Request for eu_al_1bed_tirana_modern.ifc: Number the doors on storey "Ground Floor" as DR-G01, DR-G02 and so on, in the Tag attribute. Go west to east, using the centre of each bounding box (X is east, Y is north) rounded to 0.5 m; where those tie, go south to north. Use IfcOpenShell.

First a look at what the model holds.

```python
import ifcopenshell
import ifcopenshell.util.element
import ifcopenshell.util.placement

model = ifcopenshell.open("eu_al_1bed_tirana_modern.ifc")
print(model.schema)
storey = next(s for s in model.by_type("IfcBuildingStorey") if s.Name == "Ground Floor")
doors = [e for e in ifcopenshell.util.element.get_decomposition(storey) if e.is_a("IfcDoor")]
for e in sorted(doors, key=lambda e: e.id()):
    origin = ifcopenshell.util.placement.get_local_placement(e.ObjectPlacement)[:3, 3]
    print(e.id(), e.Tag, e.Name, origin.round(2) + 0.0, sep=" | ")
```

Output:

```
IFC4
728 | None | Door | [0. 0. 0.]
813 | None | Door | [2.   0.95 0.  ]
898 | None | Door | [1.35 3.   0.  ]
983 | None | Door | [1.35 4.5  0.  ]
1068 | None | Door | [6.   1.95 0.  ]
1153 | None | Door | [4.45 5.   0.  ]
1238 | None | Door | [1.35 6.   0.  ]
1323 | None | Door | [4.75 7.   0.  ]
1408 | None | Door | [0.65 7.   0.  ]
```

```python
import ifcopenshell
import ifcopenshell.geom
import ifcopenshell.util.element
import ifcopenshell.util.shape

model = ifcopenshell.open("eu_al_1bed_tirana_modern.ifc")
settings = ifcopenshell.geom.settings()
settings.set("use-world-coords", True)


def centre(element):
    shape = ifcopenshell.geom.create_shape(settings, element)
    return ifcopenshell.util.shape.get_bbox_centroid(shape.geometry)


storey = next(s for s in model.by_type("IfcBuildingStorey") if s.Name == "Ground Floor")
doors = [e for e in ifcopenshell.util.element.get_decomposition(storey) if e.is_a("IfcDoor")]

# Insertion points can sit at a corner or the storey origin, so sort by the geometry (in metres).
centres = {e: centre(e) for e in doors}
doors.sort(key=lambda e: (round(centres[e][0] / 0.5), centres[e][1]))

for i, e in enumerate(doors, start=1):
    number = f"DR-G{i:02d}"
    e.Tag = number
    print(e.id(), number)

model.write("eu_al_1bed_tirana_modern_rev.ifc")
```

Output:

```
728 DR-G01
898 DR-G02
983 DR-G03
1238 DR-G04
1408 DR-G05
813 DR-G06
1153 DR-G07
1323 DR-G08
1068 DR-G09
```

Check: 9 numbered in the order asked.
